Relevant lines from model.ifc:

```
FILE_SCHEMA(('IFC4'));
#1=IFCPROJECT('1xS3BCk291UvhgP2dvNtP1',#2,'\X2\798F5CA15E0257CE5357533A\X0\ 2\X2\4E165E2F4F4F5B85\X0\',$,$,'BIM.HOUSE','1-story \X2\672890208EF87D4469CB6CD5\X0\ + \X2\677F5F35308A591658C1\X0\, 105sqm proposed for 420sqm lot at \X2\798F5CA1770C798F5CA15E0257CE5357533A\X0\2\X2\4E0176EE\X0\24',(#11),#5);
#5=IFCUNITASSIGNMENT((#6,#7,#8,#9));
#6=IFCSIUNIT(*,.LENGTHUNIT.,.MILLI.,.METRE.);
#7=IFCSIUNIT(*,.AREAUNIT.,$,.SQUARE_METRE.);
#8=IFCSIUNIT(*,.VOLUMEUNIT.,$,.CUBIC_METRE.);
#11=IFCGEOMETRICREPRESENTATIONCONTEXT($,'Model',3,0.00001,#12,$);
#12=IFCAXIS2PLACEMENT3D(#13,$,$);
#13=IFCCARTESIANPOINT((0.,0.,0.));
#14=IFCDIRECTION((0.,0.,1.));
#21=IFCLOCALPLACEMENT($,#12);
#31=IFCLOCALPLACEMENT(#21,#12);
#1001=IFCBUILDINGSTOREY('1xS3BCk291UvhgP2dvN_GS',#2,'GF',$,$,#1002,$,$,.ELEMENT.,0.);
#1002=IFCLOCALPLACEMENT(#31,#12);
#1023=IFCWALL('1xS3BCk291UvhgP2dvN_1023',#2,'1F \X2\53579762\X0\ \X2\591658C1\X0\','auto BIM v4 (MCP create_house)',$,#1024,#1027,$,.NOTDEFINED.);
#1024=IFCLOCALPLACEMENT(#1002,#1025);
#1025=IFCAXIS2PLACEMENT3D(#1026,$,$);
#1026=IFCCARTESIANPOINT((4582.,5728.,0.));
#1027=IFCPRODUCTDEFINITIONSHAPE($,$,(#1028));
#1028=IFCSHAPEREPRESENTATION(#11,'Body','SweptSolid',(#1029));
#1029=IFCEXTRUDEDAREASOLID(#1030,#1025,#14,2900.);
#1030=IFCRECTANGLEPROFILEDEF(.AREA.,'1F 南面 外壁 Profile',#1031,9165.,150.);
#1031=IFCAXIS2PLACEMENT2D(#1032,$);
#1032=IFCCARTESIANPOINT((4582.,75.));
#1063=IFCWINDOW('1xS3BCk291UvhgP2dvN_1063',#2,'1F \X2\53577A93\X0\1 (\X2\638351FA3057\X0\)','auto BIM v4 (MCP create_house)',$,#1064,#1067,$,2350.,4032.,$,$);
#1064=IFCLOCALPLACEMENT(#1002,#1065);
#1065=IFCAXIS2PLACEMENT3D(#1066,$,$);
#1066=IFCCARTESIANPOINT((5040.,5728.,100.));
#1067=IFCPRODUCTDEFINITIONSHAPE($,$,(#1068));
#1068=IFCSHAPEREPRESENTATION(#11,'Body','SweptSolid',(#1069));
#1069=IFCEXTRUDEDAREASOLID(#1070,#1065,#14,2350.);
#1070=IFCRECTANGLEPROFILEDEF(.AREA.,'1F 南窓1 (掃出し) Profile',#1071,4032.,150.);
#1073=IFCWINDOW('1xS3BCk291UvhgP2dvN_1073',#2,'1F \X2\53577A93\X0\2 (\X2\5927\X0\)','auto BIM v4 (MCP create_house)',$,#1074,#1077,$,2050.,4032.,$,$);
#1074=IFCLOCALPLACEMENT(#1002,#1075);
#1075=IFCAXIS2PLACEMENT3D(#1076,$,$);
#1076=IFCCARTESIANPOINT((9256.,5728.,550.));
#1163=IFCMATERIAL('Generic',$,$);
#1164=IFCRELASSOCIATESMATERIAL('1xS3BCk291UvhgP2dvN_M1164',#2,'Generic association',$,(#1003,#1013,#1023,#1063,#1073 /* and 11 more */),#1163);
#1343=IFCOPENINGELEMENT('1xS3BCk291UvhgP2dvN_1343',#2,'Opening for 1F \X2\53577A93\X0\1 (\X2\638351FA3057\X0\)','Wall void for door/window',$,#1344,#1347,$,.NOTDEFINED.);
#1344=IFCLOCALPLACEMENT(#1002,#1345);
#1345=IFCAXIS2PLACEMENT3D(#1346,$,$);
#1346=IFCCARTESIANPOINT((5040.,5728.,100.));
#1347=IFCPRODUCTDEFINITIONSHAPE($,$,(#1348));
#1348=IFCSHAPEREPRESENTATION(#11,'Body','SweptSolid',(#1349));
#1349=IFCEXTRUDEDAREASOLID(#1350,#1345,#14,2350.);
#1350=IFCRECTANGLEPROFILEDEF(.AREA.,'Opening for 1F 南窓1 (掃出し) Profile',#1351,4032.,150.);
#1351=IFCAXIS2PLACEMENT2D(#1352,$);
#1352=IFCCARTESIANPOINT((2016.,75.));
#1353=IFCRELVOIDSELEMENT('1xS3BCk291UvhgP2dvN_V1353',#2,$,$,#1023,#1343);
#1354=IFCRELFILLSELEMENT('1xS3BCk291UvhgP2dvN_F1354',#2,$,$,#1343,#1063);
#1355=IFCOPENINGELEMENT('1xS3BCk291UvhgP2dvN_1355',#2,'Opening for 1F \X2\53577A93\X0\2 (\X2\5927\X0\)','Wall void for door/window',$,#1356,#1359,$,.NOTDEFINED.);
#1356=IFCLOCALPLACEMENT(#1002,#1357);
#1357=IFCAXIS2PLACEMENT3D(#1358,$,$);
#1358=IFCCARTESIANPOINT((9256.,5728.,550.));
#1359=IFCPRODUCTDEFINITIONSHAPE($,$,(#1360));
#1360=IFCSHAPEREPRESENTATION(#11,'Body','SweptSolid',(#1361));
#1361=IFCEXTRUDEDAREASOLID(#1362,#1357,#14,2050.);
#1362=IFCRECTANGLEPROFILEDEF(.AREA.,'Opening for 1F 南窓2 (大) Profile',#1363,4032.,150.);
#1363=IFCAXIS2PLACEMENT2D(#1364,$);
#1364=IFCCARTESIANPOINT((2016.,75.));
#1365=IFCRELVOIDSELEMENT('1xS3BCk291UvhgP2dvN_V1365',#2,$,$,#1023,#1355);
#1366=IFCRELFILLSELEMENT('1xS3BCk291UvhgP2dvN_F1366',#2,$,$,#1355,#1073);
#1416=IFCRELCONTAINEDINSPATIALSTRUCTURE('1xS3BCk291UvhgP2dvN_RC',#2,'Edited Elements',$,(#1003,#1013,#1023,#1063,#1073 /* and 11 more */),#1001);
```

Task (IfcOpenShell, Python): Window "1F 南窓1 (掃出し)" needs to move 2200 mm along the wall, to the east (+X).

```python
import ifcopenshell
import ifcopenshell.api.geometry
import ifcopenshell.util.placement
import ifcopenshell.util.unit

model = ifcopenshell.open("model.ifc")
unit_scale = ifcopenshell.util.unit.calculate_unit_scale(model)

window = model.by_guid("1xS3BCk291UvhgP2dvN_1063")
opening = window.FillsVoids[0].RelatingOpeningElement
wall = opening.VoidsElements[0].RelatingBuildingElement

wall_matrix = ifcopenshell.util.placement.get_local_placement(wall.ObjectPlacement)
shift = wall_matrix[:3, 0] * 2.2 / unit_scale
before = ifcopenshell.util.placement.get_local_placement(window.ObjectPlacement)[:3, 3].copy()

# The window is not placed relative to its opening, so move both.
for product in (opening, window):
    matrix = ifcopenshell.util.placement.get_local_placement(product.ObjectPlacement)
    matrix[:3, 3] += shift
    ifcopenshell.api.geometry.edit_object_placement(model, product=product, matrix=matrix, is_si=False)

after = ifcopenshell.util.placement.get_local_placement(window.ObjectPlacement)[:3, 3]
print("window moved by", (after - before).round(3) + 0.0)

model.write("model-out.ifc")
```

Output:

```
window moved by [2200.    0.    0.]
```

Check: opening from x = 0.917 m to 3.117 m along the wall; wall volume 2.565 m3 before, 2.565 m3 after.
